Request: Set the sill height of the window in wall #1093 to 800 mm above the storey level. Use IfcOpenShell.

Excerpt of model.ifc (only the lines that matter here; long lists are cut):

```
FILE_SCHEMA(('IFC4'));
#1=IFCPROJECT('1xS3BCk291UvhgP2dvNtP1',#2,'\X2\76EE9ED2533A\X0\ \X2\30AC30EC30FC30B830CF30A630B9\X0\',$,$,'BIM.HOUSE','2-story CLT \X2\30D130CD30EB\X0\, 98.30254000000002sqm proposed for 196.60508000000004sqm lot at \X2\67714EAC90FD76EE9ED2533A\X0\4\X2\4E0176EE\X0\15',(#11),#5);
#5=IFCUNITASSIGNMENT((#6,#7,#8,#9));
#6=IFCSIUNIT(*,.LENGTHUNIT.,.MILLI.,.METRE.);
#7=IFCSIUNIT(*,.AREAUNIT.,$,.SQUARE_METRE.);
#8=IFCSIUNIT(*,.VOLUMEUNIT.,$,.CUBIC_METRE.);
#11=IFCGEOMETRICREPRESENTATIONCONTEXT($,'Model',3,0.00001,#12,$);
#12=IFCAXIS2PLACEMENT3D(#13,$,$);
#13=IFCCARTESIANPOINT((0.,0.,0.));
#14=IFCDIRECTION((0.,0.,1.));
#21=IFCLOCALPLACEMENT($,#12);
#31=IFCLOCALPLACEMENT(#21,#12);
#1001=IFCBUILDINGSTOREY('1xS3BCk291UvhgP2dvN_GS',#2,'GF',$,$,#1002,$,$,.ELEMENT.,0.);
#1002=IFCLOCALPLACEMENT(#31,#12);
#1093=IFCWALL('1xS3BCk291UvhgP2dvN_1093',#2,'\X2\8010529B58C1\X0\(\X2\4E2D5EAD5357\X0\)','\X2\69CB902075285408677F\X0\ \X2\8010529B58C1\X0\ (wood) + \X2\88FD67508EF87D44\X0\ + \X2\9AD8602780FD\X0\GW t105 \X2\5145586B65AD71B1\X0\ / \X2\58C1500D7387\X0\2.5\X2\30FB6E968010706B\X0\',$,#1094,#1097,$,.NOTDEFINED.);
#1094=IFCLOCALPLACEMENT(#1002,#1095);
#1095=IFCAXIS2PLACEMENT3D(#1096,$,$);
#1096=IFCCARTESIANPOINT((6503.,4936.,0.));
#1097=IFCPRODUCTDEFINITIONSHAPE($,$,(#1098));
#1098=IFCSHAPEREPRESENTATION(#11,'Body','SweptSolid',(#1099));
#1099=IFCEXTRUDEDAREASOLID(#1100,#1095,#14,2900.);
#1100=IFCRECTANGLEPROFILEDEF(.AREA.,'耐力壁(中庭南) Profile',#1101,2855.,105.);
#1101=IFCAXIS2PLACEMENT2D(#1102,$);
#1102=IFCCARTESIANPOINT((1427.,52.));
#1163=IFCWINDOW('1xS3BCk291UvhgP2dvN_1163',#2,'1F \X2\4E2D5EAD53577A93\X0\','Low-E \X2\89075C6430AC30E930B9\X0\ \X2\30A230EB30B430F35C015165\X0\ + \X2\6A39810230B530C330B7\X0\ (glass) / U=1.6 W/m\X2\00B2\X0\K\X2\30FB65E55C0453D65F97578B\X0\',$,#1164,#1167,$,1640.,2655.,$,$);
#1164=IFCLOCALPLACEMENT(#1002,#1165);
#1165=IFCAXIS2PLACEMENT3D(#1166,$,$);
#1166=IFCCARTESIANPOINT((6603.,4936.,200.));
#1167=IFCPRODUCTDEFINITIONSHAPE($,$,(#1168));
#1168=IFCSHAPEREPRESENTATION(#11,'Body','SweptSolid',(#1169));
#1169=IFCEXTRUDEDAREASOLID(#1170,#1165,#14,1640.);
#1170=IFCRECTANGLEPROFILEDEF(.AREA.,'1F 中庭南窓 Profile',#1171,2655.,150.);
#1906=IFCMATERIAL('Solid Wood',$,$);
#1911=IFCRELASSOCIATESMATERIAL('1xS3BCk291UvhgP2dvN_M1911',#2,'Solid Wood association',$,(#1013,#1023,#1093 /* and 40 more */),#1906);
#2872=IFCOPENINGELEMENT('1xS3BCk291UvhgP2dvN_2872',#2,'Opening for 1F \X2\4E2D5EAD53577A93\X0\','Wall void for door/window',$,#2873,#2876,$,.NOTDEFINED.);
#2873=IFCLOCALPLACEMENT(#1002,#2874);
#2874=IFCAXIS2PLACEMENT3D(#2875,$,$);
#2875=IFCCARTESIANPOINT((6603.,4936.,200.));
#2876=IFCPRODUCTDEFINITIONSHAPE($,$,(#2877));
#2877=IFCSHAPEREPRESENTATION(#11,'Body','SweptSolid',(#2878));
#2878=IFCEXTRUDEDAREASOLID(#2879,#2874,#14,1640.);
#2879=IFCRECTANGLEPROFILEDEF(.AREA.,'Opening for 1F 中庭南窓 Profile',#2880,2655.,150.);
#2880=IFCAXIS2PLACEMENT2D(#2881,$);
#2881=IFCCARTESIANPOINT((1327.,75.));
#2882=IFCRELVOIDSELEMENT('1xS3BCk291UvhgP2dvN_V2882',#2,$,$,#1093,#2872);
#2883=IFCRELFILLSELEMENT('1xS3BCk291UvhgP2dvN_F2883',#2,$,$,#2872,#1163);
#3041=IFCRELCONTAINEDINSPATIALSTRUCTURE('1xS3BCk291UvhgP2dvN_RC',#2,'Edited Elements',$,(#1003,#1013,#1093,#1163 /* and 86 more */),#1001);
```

```python
import numpy as np
import ifcopenshell
import ifcopenshell.api.geometry
import ifcopenshell.geom
import ifcopenshell.util.element
import ifcopenshell.util.placement
import ifcopenshell.util.shape
import ifcopenshell.util.unit

model = ifcopenshell.open("model.ifc")
unit_scale = ifcopenshell.util.unit.calculate_unit_scale(model)

window = model.by_id(1163)
opening = window.FillsVoids[0].RelatingOpeningElement
storey = ifcopenshell.util.element.get_container(window, ifc_class="IfcBuildingStorey")
level = ifcopenshell.util.placement.get_local_placement(storey.ObjectPlacement)[2, 3]

# The opening's origin need not be at the sill, so measure its lowest point.
shape = ifcopenshell.geom.create_shape(ifcopenshell.geom.settings(), opening)
bottom = ifcopenshell.util.shape.get_shape_bottom_elevation(shape, shape.geometry) / unit_scale
dz = level + 0.8 / unit_scale - bottom

shift = np.array([0.0, 0.0, dz])
# The window is not placed relative to its opening, so move both.
for product in (opening, window):
    matrix = ifcopenshell.util.placement.get_local_placement(product.ObjectPlacement)
    matrix[:3, 3] += shift
    ifcopenshell.api.geometry.edit_object_placement(model, product=product, matrix=matrix, is_si=False)

print(f"moved by {dz * unit_scale:+.3f} m")

model.write("model_rev.ifc")
```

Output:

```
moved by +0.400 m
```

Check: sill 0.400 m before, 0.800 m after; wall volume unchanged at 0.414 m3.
